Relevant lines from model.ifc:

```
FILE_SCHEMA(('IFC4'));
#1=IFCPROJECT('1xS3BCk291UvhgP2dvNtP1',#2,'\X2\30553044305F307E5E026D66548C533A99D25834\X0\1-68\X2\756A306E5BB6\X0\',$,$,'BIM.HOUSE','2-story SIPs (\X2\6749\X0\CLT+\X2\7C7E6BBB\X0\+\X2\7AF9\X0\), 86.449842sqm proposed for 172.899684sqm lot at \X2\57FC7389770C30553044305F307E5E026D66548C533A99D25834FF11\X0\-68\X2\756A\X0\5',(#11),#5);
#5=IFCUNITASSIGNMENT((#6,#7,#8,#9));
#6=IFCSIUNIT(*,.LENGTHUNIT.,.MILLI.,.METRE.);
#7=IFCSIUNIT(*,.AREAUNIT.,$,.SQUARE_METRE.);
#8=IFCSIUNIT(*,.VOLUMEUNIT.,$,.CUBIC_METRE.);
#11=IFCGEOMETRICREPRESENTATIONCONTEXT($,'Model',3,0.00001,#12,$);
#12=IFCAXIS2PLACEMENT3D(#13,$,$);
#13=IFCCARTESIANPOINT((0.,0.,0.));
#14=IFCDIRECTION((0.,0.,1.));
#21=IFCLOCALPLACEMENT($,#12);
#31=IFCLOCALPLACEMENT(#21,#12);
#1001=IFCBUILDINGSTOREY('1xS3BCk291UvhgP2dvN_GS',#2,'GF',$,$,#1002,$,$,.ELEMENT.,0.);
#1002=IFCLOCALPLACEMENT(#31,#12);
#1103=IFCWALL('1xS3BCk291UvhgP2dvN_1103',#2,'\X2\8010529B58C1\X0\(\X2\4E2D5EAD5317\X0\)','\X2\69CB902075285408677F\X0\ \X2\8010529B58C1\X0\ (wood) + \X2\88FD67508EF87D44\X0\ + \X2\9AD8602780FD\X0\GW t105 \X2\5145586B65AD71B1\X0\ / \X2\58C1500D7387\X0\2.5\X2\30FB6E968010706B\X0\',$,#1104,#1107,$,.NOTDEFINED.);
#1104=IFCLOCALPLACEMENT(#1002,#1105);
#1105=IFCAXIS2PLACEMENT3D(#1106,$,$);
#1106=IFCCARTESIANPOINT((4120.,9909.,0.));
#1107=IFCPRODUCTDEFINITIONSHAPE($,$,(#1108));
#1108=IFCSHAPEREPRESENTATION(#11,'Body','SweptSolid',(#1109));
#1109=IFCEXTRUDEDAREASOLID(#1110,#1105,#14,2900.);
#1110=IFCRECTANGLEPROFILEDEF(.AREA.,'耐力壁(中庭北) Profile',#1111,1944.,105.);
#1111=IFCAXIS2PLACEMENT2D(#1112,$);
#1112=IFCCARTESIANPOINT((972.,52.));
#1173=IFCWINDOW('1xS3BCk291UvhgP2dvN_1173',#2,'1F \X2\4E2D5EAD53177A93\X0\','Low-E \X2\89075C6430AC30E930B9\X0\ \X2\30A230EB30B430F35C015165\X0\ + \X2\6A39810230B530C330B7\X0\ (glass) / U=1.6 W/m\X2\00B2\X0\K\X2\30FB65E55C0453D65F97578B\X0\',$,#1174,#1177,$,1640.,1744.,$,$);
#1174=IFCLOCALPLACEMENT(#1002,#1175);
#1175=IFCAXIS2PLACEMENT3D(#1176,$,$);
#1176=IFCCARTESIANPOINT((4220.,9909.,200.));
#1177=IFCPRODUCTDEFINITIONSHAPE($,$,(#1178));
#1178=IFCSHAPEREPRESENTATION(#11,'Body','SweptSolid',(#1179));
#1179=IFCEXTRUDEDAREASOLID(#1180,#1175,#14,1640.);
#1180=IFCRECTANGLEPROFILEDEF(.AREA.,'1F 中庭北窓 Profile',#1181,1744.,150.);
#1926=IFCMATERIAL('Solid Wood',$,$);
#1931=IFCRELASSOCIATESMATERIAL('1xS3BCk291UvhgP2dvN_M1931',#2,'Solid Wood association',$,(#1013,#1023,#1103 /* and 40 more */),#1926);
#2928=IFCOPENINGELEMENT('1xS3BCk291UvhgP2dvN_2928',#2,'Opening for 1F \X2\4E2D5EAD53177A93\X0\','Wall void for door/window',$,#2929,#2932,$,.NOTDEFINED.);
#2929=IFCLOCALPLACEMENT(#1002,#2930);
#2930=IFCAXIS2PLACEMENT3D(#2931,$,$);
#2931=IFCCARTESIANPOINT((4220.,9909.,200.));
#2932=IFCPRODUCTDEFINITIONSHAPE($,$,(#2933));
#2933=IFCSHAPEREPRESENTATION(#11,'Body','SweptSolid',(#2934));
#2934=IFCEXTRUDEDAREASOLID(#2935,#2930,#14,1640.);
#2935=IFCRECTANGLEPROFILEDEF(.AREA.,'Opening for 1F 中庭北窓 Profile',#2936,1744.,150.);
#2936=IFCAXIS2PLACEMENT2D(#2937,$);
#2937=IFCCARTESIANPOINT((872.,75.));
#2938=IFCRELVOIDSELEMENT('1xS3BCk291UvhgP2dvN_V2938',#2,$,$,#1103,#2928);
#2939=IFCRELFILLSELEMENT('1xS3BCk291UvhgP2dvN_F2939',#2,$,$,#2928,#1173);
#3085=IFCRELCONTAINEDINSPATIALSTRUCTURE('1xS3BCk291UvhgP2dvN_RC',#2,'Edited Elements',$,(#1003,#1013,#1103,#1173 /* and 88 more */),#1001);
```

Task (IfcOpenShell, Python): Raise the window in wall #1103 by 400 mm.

```python
import numpy as np
import ifcopenshell
import ifcopenshell.api.geometry
import ifcopenshell.util.placement
import ifcopenshell.util.unit

model = ifcopenshell.open("model.ifc")
unit_scale = ifcopenshell.util.unit.calculate_unit_scale(model)

window = model.by_guid("1xS3BCk291UvhgP2dvN_1173")
opening = window.FillsVoids[0].RelatingOpeningElement
dz = 400.0

shift = np.array([0.0, 0.0, dz])
# The window is not placed relative to its opening, so move both.
for product in (opening, window):
    matrix = ifcopenshell.util.placement.get_local_placement(product.ObjectPlacement)
    matrix[:3, 3] += shift
    ifcopenshell.api.geometry.edit_object_placement(model, product=product, matrix=matrix, is_si=False)

print(f"moved by {dz * unit_scale:+.3f} m")

model.write("model_edited.ifc")
```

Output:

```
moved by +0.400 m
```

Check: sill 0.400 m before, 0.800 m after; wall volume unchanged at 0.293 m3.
